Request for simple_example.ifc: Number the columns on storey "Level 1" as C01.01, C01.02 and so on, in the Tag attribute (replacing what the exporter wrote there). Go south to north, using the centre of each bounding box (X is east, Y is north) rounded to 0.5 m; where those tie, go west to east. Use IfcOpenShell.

First a look at what the model holds.

```python
import ifcopenshell
import ifcopenshell.util.element
import ifcopenshell.util.placement

model = ifcopenshell.open("simple_example.ifc")
print(model.schema)
storey = next(s for s in model.by_type("IfcBuildingStorey") if s.Name == "Level 1")
columns = [e for e in ifcopenshell.util.element.get_decomposition(storey) if e.is_a("IfcColumn")]
for e in sorted(columns, key=lambda e: e.id()):
    origin = ifcopenshell.util.placement.get_local_placement(e.ObjectPlacement)[:3, 3]
    print(e.id(), e.Tag, e.Name, origin.round(2) + 0.0, sep=" | ")
```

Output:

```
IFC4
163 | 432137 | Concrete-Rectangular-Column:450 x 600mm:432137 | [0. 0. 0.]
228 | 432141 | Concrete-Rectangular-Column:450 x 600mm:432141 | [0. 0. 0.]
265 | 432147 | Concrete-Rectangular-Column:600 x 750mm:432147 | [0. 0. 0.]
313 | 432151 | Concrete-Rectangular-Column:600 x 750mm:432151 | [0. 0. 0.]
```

```python
import ifcopenshell
import ifcopenshell.geom
import ifcopenshell.util.element
import ifcopenshell.util.shape

model = ifcopenshell.open("simple_example.ifc")
settings = ifcopenshell.geom.settings()
settings.set("use-world-coords", True)


def centre(element):
    shape = ifcopenshell.geom.create_shape(settings, element)
    return ifcopenshell.util.shape.get_bbox_centroid(shape.geometry)


storey = next(s for s in model.by_type("IfcBuildingStorey") if s.Name == "Level 1")
columns = [e for e in ifcopenshell.util.element.get_decomposition(storey) if e.is_a("IfcColumn")]

# Insertion points can sit at a corner or the storey origin, so sort by the geometry (in metres).
centres = {e: centre(e) for e in columns}
columns.sort(key=lambda e: (round(centres[e][1] / 0.5), centres[e][0]))

for i, e in enumerate(columns, start=1):
    number = f"C01.{i:02d}"
    e.Tag = number
    print(e.id(), number)

model.write("simple_example_v2.ifc")
```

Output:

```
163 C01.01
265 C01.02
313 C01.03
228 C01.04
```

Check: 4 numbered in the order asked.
